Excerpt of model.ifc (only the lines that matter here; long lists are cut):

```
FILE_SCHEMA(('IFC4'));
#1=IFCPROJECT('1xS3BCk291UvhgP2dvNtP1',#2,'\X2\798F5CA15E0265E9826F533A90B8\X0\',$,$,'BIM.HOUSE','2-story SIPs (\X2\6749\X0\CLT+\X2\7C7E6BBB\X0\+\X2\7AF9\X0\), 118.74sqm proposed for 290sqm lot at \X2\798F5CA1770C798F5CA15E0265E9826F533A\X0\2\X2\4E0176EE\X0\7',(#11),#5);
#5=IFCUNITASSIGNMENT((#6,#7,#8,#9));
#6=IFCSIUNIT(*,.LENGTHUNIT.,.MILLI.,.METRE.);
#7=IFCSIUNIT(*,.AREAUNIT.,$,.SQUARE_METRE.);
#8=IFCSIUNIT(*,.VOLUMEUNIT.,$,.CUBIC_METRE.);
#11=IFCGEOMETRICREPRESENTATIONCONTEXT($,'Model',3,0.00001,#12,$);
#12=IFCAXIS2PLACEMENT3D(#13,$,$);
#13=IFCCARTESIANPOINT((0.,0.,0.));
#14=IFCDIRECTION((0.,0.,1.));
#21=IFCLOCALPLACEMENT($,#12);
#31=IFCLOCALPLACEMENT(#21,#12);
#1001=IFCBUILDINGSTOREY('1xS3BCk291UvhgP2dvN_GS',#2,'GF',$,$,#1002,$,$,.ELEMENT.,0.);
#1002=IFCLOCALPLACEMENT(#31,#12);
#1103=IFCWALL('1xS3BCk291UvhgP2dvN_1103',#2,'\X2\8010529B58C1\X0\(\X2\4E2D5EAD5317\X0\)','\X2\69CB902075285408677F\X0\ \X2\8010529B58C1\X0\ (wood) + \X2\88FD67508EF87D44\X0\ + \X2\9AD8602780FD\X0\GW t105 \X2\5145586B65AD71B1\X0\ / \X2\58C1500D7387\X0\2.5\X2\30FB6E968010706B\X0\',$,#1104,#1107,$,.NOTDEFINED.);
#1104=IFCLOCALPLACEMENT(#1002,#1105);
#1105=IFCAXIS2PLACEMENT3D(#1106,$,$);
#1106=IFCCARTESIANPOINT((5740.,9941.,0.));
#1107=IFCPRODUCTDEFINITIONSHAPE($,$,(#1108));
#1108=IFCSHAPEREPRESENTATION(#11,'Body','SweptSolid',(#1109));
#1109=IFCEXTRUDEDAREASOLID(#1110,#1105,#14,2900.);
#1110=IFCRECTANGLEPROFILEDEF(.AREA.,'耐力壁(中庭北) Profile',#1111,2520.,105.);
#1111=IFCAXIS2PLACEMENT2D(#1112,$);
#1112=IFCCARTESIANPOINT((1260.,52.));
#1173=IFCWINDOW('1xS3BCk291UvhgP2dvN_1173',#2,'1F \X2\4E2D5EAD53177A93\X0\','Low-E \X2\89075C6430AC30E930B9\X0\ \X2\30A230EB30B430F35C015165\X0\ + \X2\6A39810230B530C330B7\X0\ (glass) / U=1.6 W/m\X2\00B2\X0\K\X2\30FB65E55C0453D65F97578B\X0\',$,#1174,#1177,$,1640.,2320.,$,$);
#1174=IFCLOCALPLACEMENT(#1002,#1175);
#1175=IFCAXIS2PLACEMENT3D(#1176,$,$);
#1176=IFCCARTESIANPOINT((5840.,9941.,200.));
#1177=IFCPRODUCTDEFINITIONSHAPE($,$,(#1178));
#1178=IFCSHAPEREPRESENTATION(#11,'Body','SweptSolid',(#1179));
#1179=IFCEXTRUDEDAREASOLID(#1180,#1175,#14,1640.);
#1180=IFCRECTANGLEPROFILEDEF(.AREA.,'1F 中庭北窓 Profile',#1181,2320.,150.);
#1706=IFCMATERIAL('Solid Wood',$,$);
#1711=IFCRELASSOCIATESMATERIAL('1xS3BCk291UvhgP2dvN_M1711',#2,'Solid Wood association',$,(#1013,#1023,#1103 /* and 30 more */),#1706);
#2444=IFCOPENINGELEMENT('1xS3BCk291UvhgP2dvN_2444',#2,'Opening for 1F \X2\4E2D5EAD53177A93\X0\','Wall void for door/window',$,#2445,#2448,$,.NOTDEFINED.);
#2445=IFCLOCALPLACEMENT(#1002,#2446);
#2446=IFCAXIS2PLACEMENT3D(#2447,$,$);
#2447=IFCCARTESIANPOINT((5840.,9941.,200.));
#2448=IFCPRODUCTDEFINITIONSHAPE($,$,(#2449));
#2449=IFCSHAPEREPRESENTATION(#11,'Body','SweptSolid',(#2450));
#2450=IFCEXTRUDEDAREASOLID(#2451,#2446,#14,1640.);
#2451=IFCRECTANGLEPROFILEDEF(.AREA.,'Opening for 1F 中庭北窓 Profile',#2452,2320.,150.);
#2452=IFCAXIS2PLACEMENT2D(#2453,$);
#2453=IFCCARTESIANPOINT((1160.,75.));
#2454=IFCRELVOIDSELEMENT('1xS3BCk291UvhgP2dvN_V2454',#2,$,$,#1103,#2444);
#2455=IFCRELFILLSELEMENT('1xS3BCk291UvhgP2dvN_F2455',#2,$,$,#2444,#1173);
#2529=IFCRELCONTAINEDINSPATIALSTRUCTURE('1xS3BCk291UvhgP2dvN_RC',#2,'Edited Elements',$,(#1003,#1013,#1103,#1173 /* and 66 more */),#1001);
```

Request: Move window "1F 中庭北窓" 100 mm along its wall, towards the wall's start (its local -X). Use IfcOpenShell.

```python
import ifcopenshell
import ifcopenshell.api.geometry
import ifcopenshell.util.placement

model = ifcopenshell.open("model.ifc")

window = model.by_guid("1xS3BCk291UvhgP2dvN_1173")
opening = window.FillsVoids[0].RelatingOpeningElement
wall = opening.VoidsElements[0].RelatingBuildingElement

wall_matrix = ifcopenshell.util.placement.get_local_placement(wall.ObjectPlacement)
shift = wall_matrix[:3, 0] * -100.0
before = ifcopenshell.util.placement.get_local_placement(window.ObjectPlacement)[:3, 3].copy()

# The window is not placed relative to its opening, so move both.
for product in (opening, window):
    matrix = ifcopenshell.util.placement.get_local_placement(product.ObjectPlacement)
    matrix[:3, 3] += shift
    ifcopenshell.api.geometry.edit_object_placement(model, product=product, matrix=matrix, is_si=False)

after = ifcopenshell.util.placement.get_local_placement(window.ObjectPlacement)[:3, 3]
print("window moved by", (after - before).round(3) + 0.0)

model.write("model_updated.ifc")
```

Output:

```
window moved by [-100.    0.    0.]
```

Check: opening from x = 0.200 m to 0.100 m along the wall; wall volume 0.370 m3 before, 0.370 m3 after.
